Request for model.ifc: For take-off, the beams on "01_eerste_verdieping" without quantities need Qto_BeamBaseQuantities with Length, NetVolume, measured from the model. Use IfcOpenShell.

First a look at what the model holds.

```python
import ifcopenshell
import ifcopenshell.util.element
import ifcopenshell.util.unit

model = ifcopenshell.open("model.ifc")
print(model.schema)
for unit_type in ("LENGTHUNIT", "AREAUNIT", "VOLUMEUNIT"):
    print(unit_type, ifcopenshell.util.unit.calculate_unit_scale(model, unit_type))
storey = next(s for s in model.by_type("IfcBuildingStorey") if s.Name == "01_eerste_verdieping")
beams = [e for e in ifcopenshell.util.element.get_decomposition(storey) if e.is_a("IfcBeam")]
for e in sorted(beams, key=lambda e: e.id()):
    print(e.id(), e.is_a(), e.Name, list(ifcopenshell.util.element.get_psets(e, qtos_only=True)), sep=" | ")
```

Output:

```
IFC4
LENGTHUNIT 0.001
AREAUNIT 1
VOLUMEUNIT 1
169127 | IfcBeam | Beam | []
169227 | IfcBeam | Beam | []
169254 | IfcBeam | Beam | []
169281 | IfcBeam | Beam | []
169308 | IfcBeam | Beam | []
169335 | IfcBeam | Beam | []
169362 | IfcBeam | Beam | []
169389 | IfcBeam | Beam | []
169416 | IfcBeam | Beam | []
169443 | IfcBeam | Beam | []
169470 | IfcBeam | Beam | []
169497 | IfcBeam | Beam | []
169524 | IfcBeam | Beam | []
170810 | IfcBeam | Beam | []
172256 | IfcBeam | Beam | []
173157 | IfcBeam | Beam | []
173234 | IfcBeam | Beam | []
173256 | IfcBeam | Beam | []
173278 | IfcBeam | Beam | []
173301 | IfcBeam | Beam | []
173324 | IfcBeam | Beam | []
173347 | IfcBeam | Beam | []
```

```python
import ifcopenshell
import ifcopenshell.api.pset
import ifcopenshell.geom
import ifcopenshell.util.element
import ifcopenshell.util.shape
import ifcopenshell.util.unit

model = ifcopenshell.open("model.ifc")
unit_scale = ifcopenshell.util.unit.calculate_unit_scale(model)
volume_scale = ifcopenshell.util.unit.calculate_unit_scale(model, "VOLUMEUNIT")
settings = ifcopenshell.geom.settings()

storey = next(s for s in model.by_type("IfcBuildingStorey") if s.Name == "01_eerste_verdieping")
beams = [e for e in ifcopenshell.util.element.get_decomposition(storey) if e.is_a("IfcBeam")]

for e in sorted(beams, key=lambda e: e.id()):
    if ifcopenshell.util.element.get_psets(e, qtos_only=True, should_inherit=False):
        continue
    # Geometry comes back in metres, in the element's own axes.
    shape = ifcopenshell.geom.create_shape(settings, e)
    values = {
        "Length": ifcopenshell.util.shape.get_max_xyz(shape.geometry) / unit_scale,
        "NetVolume": ifcopenshell.util.shape.get_volume(shape.geometry) / volume_scale,
    }
    qto = ifcopenshell.api.pset.add_qto(model, product=e, name="Qto_BeamBaseQuantities")
    ifcopenshell.api.pset.edit_qto(model, qto=qto, properties=values)
    print(e.id(), {k: round(v, 3) for k, v in values.items()})

model.write("model_updated.ifc")
```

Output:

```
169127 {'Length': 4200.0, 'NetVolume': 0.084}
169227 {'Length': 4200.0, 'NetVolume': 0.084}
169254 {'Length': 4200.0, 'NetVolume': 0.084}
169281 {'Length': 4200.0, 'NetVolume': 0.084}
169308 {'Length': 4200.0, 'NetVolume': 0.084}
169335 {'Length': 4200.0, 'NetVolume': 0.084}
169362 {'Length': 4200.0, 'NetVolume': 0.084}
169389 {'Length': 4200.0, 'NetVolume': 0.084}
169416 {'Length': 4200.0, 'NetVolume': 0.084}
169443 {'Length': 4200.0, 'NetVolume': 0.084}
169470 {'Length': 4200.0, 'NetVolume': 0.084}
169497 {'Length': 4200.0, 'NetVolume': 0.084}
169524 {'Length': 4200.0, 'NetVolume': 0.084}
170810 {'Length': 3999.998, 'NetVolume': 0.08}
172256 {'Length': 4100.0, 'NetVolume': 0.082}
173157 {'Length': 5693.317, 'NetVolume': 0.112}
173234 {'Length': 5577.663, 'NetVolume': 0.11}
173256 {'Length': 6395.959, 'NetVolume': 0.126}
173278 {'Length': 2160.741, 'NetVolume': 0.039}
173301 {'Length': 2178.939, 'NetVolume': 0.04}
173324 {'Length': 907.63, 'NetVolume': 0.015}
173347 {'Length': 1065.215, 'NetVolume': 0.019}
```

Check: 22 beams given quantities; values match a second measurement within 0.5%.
